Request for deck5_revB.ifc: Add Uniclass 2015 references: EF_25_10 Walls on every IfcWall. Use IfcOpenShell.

First a look at what the model holds.

```python
import ifcopenshell

model = ifcopenshell.open("deck5_revB.ifc")
print(model.schema)
print("classifications:", [c.Name for c in model.by_type("IfcClassification")])
for ifc_class in ("IfcDoor", "IfcRoof", "IfcStair", "IfcWall", "IfcWindow"):
    print(ifc_class, len(model.by_type(ifc_class)))
```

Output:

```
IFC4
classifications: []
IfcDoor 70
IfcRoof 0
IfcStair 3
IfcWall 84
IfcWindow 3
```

```python
import ifcopenshell
import ifcopenshell.api.classification

model = ifcopenshell.open("deck5_revB.ifc")

system = ifcopenshell.api.classification.add_classification(model, classification="Uniclass 2015")

codes = {
    "IfcWall": ("EF_25_10", "Walls"),
}
for ifc_class, (code, name) in codes.items():
    products = model.by_type(ifc_class)
    ifcopenshell.api.classification.add_reference(
        model, products=products, classification=system, identification=code, name=name
    )
    print(code, len(products))

model.write("deck5_revB_v2.ifc")
```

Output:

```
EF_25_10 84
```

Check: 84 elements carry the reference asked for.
